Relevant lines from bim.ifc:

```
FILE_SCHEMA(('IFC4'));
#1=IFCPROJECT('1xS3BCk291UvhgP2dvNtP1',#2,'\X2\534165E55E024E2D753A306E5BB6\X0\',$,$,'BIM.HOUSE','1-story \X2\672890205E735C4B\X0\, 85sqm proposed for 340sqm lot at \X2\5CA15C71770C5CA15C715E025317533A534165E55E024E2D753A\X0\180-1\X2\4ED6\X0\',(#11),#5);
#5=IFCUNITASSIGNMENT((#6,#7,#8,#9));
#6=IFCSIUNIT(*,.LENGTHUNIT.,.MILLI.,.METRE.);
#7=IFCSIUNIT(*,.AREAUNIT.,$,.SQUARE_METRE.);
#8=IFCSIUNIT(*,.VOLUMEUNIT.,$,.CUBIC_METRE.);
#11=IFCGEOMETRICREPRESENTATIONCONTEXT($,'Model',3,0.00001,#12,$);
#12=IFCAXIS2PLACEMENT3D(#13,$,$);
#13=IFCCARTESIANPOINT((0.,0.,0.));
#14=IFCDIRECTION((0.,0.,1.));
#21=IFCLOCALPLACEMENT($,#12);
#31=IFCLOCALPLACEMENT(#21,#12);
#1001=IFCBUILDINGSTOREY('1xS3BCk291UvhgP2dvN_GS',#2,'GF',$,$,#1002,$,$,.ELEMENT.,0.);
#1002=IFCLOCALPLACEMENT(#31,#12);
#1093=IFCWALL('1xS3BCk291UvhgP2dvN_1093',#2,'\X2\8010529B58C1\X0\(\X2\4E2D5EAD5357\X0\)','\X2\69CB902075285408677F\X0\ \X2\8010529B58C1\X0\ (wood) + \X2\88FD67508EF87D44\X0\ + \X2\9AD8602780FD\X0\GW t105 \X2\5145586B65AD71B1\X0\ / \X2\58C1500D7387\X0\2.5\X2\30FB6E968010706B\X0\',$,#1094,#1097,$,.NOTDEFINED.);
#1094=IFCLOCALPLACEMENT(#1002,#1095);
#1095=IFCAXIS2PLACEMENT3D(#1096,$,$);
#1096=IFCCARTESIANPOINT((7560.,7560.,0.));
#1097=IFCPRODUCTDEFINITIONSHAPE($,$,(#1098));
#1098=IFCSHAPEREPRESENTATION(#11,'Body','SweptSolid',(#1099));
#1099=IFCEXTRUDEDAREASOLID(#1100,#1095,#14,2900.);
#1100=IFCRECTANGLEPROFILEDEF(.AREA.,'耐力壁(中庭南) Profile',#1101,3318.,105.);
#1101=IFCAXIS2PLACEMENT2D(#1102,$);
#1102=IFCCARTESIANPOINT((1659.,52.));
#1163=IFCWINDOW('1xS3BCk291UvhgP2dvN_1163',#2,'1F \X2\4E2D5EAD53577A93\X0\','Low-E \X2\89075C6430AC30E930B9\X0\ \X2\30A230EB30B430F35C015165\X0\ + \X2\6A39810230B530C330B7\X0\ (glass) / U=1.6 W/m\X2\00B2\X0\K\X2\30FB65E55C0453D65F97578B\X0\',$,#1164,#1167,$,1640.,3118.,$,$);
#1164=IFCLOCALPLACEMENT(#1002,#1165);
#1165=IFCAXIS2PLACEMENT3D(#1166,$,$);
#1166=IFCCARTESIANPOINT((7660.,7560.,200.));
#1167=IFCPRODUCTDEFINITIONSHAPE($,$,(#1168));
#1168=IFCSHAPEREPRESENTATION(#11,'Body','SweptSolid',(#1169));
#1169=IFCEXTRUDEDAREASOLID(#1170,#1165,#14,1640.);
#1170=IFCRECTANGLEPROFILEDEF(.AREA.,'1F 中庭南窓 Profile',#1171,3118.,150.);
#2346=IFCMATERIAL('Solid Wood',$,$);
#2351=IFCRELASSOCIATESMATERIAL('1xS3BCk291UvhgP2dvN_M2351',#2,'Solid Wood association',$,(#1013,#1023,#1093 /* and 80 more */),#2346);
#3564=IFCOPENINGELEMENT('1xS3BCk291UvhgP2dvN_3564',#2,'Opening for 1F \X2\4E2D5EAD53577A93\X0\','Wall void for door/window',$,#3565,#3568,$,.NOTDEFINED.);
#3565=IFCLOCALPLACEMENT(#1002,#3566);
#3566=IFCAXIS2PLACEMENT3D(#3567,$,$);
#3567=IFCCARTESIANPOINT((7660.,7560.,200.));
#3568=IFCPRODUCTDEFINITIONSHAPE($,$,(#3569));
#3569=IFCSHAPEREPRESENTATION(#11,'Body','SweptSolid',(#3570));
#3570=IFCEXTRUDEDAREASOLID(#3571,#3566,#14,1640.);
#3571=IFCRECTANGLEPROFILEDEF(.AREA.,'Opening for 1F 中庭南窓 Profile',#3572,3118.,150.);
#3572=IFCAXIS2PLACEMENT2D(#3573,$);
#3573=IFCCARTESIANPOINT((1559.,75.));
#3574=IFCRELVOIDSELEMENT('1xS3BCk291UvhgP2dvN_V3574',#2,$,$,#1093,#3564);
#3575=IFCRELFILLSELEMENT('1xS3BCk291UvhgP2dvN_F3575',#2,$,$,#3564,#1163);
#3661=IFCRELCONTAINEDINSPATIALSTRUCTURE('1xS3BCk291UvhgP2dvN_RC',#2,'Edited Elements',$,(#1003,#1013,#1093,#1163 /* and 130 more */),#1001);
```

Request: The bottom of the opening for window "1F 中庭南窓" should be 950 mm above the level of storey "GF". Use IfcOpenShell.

```python
import numpy as np
import ifcopenshell
import ifcopenshell.api.geometry
import ifcopenshell.geom
import ifcopenshell.util.element
import ifcopenshell.util.placement
import ifcopenshell.util.shape
import ifcopenshell.util.unit

model = ifcopenshell.open("bim.ifc")
unit_scale = ifcopenshell.util.unit.calculate_unit_scale(model)

window = model.by_guid("1xS3BCk291UvhgP2dvN_1163")
opening = window.FillsVoids[0].RelatingOpeningElement
storey = ifcopenshell.util.element.get_container(window, ifc_class="IfcBuildingStorey")
level = ifcopenshell.util.placement.get_local_placement(storey.ObjectPlacement)[2, 3]

# The opening's origin need not be at the sill, so measure its lowest point.
shape = ifcopenshell.geom.create_shape(ifcopenshell.geom.settings(), opening)
bottom = ifcopenshell.util.shape.get_shape_bottom_elevation(shape, shape.geometry) / unit_scale
dz = level + 950.0 - bottom

shift = np.array([0.0, 0.0, dz])
# The window is not placed relative to its opening, so move both.
for product in (opening, window):
    matrix = ifcopenshell.util.placement.get_local_placement(product.ObjectPlacement)
    matrix[:3, 3] += shift
    ifcopenshell.api.geometry.edit_object_placement(model, product=product, matrix=matrix, is_si=False)

print(f"moved by {dz * unit_scale:+.3f} m")

model.write("bim_updated.ifc")
```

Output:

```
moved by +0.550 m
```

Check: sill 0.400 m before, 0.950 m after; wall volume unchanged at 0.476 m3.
